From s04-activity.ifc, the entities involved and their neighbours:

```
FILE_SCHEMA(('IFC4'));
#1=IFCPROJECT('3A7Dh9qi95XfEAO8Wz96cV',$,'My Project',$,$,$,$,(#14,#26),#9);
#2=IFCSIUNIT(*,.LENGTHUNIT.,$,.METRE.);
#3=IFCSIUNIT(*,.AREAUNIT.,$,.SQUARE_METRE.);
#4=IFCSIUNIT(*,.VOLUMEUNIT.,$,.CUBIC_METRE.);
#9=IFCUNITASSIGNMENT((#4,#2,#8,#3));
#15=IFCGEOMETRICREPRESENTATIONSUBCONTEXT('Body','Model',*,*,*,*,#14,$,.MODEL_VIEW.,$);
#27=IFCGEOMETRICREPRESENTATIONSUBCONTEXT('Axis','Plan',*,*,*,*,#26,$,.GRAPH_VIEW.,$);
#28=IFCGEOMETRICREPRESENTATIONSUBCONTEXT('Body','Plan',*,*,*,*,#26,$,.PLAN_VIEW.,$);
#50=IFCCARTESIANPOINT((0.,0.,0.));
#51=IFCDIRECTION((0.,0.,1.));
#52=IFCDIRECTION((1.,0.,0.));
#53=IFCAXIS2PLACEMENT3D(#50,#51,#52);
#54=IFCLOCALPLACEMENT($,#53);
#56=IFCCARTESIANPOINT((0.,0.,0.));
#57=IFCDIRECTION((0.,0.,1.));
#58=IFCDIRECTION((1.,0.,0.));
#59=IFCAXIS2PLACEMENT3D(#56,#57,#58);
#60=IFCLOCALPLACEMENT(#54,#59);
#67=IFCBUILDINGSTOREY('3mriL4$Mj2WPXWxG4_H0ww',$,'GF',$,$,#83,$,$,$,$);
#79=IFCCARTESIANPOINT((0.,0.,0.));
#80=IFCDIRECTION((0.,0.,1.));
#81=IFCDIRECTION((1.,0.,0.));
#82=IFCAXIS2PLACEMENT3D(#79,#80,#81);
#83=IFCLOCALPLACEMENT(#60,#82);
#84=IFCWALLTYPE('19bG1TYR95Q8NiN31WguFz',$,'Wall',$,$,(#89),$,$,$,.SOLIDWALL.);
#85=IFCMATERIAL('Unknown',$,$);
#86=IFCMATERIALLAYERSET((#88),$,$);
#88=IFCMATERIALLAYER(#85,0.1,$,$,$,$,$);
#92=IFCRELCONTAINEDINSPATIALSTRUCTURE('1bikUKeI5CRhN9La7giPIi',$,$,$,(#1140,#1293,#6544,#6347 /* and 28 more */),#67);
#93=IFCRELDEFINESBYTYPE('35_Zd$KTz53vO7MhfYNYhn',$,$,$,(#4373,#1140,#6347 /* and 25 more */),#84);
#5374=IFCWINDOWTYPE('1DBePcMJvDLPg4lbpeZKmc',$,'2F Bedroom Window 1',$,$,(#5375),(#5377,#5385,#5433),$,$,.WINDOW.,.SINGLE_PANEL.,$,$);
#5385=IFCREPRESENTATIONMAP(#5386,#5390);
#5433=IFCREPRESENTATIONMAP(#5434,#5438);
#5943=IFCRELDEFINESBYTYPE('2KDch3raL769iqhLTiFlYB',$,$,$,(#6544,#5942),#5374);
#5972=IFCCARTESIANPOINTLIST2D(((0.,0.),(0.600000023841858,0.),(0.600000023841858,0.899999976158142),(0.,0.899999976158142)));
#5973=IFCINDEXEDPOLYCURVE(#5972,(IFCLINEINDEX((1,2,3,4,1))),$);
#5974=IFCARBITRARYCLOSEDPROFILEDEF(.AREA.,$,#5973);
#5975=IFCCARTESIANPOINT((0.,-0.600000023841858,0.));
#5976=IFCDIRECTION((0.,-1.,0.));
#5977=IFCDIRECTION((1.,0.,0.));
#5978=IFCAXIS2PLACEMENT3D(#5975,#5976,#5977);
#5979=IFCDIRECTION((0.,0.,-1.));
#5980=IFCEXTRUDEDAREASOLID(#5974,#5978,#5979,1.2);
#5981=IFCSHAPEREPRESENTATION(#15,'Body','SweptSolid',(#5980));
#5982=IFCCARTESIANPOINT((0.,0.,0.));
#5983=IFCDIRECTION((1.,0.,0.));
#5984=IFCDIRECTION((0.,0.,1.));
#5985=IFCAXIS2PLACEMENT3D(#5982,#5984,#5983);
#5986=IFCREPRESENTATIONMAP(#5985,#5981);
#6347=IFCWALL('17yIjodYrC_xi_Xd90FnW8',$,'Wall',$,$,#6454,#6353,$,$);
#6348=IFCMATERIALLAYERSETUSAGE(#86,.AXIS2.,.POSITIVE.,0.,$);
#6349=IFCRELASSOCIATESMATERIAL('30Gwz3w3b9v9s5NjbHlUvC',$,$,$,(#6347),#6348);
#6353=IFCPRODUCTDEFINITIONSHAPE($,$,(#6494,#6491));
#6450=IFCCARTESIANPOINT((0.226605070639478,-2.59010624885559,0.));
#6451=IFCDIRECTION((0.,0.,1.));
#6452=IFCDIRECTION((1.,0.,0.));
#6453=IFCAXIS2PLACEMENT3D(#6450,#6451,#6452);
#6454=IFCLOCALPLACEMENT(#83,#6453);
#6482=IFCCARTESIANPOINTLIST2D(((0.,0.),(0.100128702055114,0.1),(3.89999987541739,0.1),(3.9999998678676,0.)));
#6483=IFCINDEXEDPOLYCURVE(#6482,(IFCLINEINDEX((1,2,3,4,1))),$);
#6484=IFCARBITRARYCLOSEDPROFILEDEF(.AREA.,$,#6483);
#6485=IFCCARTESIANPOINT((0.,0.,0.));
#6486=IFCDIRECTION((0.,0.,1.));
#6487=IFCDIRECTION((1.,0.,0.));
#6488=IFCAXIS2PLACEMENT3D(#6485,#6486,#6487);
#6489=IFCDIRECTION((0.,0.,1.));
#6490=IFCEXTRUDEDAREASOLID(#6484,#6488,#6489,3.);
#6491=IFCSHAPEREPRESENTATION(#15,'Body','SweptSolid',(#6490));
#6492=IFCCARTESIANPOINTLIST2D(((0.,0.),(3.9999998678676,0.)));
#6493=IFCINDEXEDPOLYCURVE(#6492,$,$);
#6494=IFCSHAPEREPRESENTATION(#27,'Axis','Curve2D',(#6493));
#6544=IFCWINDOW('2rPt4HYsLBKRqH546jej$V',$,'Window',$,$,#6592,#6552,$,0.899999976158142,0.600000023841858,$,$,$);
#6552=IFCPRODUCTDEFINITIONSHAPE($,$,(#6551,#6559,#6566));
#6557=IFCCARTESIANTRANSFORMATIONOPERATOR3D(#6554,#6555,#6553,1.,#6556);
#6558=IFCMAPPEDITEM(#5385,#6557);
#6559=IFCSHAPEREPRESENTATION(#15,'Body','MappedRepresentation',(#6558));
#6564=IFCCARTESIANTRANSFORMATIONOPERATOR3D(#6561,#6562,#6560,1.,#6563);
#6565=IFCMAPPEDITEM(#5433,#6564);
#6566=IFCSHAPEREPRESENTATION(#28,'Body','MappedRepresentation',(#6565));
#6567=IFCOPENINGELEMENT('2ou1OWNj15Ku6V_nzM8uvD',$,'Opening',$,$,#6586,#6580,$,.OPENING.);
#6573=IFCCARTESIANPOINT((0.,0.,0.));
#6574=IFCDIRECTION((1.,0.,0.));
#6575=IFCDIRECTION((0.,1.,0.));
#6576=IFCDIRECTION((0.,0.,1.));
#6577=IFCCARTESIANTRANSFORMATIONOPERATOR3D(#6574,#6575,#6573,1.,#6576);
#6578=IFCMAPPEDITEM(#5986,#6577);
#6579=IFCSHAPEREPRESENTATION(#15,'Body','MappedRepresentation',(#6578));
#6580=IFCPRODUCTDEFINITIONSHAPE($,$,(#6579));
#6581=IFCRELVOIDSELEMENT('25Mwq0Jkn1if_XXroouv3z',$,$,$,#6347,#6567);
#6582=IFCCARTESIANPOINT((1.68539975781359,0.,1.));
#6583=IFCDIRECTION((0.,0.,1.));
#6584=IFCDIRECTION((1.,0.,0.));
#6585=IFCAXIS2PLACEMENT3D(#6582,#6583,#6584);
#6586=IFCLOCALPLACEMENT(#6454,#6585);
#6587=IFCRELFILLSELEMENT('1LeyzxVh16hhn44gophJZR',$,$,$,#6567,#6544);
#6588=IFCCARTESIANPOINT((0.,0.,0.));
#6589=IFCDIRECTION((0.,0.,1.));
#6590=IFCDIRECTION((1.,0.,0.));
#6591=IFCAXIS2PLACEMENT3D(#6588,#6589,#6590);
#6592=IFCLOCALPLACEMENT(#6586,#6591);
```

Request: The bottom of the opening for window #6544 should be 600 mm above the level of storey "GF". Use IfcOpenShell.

```python
import numpy as np
import ifcopenshell
import ifcopenshell.api.geometry
import ifcopenshell.geom
import ifcopenshell.util.element
import ifcopenshell.util.placement
import ifcopenshell.util.shape
import ifcopenshell.util.unit

model = ifcopenshell.open("s04-activity.ifc")
unit_scale = ifcopenshell.util.unit.calculate_unit_scale(model)

window = model.by_id(6544)
opening = window.FillsVoids[0].RelatingOpeningElement
storey = ifcopenshell.util.element.get_container(window, ifc_class="IfcBuildingStorey")
level = ifcopenshell.util.placement.get_local_placement(storey.ObjectPlacement)[2, 3]

# The opening's origin need not be at the sill, so measure its lowest point.
shape = ifcopenshell.geom.create_shape(ifcopenshell.geom.settings(), opening)
bottom = ifcopenshell.util.shape.get_shape_bottom_elevation(shape, shape.geometry) / unit_scale
dz = level + 0.6 - bottom

shift = np.array([0.0, 0.0, dz])
# The window is placed relative to its opening, so it follows when the opening moves.
matrix = ifcopenshell.util.placement.get_local_placement(opening.ObjectPlacement)
matrix[:3, 3] += shift
ifcopenshell.api.geometry.edit_object_placement(
    model, product=opening, matrix=matrix, is_si=False, should_transform_children=True
)

print(f"moved by {dz * unit_scale:+.3f} m")

model.write("s04-activity_updated.ifc")
```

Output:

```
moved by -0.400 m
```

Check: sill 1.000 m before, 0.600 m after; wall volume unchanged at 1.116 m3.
